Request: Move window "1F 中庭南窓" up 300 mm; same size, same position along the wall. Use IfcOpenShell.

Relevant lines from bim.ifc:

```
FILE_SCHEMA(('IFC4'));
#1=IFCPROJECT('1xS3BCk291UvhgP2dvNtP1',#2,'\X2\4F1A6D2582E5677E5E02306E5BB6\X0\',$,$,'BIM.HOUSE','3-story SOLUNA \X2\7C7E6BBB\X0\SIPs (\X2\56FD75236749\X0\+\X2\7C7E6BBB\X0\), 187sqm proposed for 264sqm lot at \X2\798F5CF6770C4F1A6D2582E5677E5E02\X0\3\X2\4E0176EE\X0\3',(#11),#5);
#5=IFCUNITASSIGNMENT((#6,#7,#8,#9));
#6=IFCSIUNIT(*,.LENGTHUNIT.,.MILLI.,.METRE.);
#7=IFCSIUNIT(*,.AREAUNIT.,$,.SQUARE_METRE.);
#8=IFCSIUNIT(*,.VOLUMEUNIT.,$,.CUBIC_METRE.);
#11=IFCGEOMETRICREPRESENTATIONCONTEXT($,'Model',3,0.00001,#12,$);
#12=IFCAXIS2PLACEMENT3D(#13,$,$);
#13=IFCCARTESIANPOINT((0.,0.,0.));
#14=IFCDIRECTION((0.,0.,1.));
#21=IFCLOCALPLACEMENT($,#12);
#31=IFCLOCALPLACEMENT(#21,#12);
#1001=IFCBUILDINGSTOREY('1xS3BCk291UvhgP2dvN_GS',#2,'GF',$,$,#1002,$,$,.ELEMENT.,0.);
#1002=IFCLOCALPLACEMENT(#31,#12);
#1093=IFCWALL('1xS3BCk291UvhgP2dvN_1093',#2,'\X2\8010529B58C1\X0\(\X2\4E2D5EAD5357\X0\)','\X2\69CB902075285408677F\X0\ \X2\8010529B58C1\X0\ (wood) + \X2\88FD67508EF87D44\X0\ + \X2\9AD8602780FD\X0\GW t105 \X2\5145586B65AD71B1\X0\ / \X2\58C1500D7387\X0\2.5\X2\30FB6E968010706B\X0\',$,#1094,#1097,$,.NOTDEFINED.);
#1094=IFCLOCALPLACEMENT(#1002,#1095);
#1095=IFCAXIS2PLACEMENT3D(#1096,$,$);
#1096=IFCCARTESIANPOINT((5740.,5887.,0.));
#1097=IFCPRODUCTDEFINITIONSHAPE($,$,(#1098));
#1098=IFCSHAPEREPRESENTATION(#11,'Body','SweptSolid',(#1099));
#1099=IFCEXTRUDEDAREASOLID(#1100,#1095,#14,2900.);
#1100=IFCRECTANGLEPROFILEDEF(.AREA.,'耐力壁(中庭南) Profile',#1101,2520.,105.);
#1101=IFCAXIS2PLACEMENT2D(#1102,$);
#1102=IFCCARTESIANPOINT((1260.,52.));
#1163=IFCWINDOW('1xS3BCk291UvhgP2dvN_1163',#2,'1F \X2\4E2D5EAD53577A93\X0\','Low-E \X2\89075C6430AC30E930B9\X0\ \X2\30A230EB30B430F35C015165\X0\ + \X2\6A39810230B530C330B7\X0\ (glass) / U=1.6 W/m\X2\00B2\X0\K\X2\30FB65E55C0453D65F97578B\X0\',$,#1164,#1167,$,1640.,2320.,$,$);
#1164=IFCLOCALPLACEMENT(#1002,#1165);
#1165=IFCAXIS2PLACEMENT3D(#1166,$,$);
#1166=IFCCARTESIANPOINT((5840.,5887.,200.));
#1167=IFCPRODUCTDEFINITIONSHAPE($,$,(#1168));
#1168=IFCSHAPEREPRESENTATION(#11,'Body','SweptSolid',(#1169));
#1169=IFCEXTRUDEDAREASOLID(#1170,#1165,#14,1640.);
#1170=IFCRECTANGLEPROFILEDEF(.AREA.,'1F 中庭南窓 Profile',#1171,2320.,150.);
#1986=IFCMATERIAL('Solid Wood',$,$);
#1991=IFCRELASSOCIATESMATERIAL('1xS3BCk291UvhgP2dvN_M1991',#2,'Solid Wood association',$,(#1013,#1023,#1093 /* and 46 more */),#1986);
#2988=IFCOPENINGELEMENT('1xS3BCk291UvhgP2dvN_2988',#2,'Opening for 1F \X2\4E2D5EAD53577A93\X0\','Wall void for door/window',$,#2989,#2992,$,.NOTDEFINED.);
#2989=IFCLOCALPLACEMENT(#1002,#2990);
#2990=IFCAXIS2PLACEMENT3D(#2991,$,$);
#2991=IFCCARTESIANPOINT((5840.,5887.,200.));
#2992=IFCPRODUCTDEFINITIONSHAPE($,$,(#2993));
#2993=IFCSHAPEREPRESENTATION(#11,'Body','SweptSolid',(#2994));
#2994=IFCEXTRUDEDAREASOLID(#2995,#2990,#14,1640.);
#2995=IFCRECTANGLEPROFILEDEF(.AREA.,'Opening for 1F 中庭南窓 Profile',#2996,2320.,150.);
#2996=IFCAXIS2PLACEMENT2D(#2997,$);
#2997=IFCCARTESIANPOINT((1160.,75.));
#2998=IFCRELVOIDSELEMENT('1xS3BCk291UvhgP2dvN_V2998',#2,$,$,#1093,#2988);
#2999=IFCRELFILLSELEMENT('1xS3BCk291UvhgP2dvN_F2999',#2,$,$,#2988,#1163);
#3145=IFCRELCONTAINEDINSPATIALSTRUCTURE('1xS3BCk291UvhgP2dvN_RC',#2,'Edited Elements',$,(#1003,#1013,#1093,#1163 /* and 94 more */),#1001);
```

```python
import numpy as np
import ifcopenshell
import ifcopenshell.api.geometry
import ifcopenshell.util.placement
import ifcopenshell.util.unit

model = ifcopenshell.open("bim.ifc")
unit_scale = ifcopenshell.util.unit.calculate_unit_scale(model)

window = model.by_guid("1xS3BCk291UvhgP2dvN_1163")
opening = window.FillsVoids[0].RelatingOpeningElement
dz = 300.0

shift = np.array([0.0, 0.0, dz])
# The window is not placed relative to its opening, so move both.
for product in (opening, window):
    matrix = ifcopenshell.util.placement.get_local_placement(product.ObjectPlacement)
    matrix[:3, 3] += shift
    ifcopenshell.api.geometry.edit_object_placement(model, product=product, matrix=matrix, is_si=False)

print(f"moved by {dz * unit_scale:+.3f} m")

model.write("bim-out.ifc")
```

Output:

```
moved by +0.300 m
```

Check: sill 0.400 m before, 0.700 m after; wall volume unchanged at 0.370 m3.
